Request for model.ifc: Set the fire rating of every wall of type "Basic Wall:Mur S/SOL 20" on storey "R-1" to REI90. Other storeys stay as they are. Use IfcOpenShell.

First a look at what the model holds.

```python
import ifcopenshell
import ifcopenshell.util.element

model = ifcopenshell.open("model.ifc")
print(model.schema)
storey = next(s for s in model.by_type("IfcBuildingStorey") if s.Name == "R-1")
walls = [e for e in ifcopenshell.util.element.get_decomposition(storey) if e.is_a("IfcWall")]
seen = {}
for e in walls:
    element_type = ifcopenshell.util.element.get_type(e)
    key = (element_type.Name if element_type != e and element_type else None, ifcopenshell.util.element.get_pset(e, "Pset_WallCommon", "FireRating"))
    seen[key] = seen.get(key, 0) + 1
for (name, value), count in sorted(seen.items(), key=str):
    print(count, "x", name, "|", value)
```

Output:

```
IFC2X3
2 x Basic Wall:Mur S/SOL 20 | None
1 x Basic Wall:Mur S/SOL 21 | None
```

```python
import ifcopenshell
import ifcopenshell.api.pset
import ifcopenshell.util.element

model = ifcopenshell.open("model.ifc")

storey = next(s for s in model.by_type("IfcBuildingStorey") if s.Name == "R-1")
walls = [e for e in ifcopenshell.util.element.get_decomposition(storey) if e.is_a("IfcWall")]

count = 0
for e in walls:
    element_type = ifcopenshell.util.element.get_type(e)
    if element_type in (None, e) or element_type.Name != "Basic Wall:Mur S/SOL 20":
        continue
    # add_pset returns the element's existing set when there is one.
    pset = ifcopenshell.api.pset.add_pset(model, product=e, name="Pset_WallCommon")
    ifcopenshell.api.pset.edit_pset(model, pset=pset, properties={"FireRating": "REI90"})
    count += 1

print(count, "walls updated")

model.write("model_rev.ifc")
```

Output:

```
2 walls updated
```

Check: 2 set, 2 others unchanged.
